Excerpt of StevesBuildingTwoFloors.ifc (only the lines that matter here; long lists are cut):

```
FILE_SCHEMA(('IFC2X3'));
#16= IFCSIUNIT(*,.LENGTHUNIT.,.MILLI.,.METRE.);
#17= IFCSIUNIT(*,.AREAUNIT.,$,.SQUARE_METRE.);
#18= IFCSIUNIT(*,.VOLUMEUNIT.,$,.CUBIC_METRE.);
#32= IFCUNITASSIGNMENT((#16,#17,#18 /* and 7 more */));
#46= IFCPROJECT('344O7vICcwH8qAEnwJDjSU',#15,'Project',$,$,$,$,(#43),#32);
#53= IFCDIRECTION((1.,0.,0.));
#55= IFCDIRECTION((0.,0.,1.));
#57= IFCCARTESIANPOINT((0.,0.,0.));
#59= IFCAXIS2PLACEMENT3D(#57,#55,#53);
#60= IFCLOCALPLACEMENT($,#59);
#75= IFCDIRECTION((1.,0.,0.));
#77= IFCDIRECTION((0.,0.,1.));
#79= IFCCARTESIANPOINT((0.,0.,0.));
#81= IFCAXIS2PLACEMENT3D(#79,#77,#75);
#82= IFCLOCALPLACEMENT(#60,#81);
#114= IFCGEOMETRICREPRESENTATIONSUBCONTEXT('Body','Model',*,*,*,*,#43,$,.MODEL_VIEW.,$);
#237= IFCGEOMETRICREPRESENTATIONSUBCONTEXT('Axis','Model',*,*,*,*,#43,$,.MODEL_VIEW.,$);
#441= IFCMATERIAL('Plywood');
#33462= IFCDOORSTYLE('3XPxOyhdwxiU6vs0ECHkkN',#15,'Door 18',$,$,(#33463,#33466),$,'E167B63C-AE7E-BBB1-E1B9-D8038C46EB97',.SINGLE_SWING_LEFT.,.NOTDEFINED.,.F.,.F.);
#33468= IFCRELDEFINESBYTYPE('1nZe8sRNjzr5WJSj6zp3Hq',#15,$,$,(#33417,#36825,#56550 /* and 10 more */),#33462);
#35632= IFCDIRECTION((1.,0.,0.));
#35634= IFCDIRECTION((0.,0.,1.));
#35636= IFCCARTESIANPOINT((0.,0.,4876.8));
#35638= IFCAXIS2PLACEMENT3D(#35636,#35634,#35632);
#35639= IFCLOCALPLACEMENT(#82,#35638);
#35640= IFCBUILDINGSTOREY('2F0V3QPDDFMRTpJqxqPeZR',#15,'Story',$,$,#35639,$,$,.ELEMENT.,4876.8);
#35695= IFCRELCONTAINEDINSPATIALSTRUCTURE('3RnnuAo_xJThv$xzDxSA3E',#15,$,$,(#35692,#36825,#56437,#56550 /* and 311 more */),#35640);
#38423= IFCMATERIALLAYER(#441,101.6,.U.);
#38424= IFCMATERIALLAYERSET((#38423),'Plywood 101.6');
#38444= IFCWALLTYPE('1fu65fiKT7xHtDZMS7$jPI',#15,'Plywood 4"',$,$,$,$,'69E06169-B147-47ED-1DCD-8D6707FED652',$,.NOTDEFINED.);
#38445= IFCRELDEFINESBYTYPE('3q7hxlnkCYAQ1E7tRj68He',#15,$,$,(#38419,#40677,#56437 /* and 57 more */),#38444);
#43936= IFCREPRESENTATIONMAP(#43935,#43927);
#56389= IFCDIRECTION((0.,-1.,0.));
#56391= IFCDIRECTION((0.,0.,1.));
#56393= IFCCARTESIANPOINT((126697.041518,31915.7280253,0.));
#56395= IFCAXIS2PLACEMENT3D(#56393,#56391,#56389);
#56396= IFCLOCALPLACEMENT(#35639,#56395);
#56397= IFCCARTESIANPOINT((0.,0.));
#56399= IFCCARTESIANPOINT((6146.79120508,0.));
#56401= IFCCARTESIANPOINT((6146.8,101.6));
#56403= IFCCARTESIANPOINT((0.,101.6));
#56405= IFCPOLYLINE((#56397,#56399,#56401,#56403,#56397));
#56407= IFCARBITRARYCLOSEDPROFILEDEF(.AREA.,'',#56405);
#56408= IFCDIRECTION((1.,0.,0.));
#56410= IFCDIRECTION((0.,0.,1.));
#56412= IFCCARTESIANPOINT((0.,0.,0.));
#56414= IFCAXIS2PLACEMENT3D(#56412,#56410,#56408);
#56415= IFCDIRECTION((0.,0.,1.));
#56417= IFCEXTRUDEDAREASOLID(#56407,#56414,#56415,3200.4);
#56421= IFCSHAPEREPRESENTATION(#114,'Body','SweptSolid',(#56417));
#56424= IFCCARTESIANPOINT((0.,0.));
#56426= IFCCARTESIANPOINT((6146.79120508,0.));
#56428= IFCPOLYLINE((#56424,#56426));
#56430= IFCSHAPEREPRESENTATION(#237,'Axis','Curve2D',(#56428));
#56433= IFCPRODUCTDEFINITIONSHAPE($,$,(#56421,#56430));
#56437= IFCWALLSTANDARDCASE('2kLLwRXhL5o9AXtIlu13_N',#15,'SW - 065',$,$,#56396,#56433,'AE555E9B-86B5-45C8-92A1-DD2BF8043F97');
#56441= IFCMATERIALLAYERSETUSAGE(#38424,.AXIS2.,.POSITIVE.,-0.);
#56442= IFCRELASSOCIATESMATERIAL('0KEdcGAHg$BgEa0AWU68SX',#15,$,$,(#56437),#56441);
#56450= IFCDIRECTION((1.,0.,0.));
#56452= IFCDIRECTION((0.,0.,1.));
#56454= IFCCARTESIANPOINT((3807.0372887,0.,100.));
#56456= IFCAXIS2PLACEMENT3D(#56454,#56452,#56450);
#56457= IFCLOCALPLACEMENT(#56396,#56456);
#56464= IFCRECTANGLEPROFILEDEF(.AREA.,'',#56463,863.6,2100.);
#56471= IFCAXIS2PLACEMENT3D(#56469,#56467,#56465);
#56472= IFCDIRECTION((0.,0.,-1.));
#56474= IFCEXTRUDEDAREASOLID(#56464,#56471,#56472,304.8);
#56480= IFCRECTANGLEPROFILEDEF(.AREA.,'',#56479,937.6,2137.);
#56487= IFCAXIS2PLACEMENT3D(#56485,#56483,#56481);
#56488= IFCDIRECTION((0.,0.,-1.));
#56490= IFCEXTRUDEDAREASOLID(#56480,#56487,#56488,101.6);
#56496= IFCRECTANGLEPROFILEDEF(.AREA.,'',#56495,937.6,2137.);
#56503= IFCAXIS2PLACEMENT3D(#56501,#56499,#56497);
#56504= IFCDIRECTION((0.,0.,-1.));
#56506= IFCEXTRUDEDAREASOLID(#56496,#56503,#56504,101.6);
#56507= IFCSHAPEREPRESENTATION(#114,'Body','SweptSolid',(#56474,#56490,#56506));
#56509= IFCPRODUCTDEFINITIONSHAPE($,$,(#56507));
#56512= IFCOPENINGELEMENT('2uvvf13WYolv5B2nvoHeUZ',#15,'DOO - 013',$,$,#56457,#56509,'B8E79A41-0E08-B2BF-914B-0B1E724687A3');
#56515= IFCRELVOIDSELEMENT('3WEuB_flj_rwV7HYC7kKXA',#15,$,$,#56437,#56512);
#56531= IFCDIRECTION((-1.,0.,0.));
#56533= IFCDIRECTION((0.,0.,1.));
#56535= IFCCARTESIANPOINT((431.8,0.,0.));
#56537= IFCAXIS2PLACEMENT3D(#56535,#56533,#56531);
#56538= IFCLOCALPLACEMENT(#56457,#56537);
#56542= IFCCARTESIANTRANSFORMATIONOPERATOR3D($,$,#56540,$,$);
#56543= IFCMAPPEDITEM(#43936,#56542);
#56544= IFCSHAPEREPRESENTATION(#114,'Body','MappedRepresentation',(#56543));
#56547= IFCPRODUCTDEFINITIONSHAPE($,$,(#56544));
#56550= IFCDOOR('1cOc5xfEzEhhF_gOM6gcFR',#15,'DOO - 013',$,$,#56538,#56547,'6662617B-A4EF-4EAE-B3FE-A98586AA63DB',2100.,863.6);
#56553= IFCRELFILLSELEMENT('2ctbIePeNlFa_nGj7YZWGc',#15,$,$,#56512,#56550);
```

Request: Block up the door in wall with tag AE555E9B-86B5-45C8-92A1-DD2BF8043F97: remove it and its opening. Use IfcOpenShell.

```python
import ifcopenshell
import ifcopenshell.api.feature
import ifcopenshell.api.root
import ifcopenshell.geom
import ifcopenshell.util.shape

model = ifcopenshell.open("StevesBuildingTwoFloors.ifc")
settings = ifcopenshell.geom.settings()


def volume(element):
    """Net volume in cubic metres, openings subtracted."""
    shape = ifcopenshell.geom.create_shape(settings, element)
    return ifcopenshell.util.shape.get_volume(shape.geometry)


door = model.by_guid("1cOc5xfEzEhhF_gOM6gcFR")
opening = door.FillsVoids[0].RelatingOpeningElement
wall = opening.VoidsElements[0].RelatingBuildingElement
before = volume(wall)

ifcopenshell.api.root.remove_product(model, product=door)
ifcopenshell.api.feature.remove_feature(model, feature=opening)

after = volume(wall)

print(f"wall volume {before:.3f} -> {after:.3f} m3")

model.write("StevesBuildingTwoFloors_edited.ifc")
```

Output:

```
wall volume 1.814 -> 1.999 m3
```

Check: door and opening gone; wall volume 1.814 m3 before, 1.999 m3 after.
